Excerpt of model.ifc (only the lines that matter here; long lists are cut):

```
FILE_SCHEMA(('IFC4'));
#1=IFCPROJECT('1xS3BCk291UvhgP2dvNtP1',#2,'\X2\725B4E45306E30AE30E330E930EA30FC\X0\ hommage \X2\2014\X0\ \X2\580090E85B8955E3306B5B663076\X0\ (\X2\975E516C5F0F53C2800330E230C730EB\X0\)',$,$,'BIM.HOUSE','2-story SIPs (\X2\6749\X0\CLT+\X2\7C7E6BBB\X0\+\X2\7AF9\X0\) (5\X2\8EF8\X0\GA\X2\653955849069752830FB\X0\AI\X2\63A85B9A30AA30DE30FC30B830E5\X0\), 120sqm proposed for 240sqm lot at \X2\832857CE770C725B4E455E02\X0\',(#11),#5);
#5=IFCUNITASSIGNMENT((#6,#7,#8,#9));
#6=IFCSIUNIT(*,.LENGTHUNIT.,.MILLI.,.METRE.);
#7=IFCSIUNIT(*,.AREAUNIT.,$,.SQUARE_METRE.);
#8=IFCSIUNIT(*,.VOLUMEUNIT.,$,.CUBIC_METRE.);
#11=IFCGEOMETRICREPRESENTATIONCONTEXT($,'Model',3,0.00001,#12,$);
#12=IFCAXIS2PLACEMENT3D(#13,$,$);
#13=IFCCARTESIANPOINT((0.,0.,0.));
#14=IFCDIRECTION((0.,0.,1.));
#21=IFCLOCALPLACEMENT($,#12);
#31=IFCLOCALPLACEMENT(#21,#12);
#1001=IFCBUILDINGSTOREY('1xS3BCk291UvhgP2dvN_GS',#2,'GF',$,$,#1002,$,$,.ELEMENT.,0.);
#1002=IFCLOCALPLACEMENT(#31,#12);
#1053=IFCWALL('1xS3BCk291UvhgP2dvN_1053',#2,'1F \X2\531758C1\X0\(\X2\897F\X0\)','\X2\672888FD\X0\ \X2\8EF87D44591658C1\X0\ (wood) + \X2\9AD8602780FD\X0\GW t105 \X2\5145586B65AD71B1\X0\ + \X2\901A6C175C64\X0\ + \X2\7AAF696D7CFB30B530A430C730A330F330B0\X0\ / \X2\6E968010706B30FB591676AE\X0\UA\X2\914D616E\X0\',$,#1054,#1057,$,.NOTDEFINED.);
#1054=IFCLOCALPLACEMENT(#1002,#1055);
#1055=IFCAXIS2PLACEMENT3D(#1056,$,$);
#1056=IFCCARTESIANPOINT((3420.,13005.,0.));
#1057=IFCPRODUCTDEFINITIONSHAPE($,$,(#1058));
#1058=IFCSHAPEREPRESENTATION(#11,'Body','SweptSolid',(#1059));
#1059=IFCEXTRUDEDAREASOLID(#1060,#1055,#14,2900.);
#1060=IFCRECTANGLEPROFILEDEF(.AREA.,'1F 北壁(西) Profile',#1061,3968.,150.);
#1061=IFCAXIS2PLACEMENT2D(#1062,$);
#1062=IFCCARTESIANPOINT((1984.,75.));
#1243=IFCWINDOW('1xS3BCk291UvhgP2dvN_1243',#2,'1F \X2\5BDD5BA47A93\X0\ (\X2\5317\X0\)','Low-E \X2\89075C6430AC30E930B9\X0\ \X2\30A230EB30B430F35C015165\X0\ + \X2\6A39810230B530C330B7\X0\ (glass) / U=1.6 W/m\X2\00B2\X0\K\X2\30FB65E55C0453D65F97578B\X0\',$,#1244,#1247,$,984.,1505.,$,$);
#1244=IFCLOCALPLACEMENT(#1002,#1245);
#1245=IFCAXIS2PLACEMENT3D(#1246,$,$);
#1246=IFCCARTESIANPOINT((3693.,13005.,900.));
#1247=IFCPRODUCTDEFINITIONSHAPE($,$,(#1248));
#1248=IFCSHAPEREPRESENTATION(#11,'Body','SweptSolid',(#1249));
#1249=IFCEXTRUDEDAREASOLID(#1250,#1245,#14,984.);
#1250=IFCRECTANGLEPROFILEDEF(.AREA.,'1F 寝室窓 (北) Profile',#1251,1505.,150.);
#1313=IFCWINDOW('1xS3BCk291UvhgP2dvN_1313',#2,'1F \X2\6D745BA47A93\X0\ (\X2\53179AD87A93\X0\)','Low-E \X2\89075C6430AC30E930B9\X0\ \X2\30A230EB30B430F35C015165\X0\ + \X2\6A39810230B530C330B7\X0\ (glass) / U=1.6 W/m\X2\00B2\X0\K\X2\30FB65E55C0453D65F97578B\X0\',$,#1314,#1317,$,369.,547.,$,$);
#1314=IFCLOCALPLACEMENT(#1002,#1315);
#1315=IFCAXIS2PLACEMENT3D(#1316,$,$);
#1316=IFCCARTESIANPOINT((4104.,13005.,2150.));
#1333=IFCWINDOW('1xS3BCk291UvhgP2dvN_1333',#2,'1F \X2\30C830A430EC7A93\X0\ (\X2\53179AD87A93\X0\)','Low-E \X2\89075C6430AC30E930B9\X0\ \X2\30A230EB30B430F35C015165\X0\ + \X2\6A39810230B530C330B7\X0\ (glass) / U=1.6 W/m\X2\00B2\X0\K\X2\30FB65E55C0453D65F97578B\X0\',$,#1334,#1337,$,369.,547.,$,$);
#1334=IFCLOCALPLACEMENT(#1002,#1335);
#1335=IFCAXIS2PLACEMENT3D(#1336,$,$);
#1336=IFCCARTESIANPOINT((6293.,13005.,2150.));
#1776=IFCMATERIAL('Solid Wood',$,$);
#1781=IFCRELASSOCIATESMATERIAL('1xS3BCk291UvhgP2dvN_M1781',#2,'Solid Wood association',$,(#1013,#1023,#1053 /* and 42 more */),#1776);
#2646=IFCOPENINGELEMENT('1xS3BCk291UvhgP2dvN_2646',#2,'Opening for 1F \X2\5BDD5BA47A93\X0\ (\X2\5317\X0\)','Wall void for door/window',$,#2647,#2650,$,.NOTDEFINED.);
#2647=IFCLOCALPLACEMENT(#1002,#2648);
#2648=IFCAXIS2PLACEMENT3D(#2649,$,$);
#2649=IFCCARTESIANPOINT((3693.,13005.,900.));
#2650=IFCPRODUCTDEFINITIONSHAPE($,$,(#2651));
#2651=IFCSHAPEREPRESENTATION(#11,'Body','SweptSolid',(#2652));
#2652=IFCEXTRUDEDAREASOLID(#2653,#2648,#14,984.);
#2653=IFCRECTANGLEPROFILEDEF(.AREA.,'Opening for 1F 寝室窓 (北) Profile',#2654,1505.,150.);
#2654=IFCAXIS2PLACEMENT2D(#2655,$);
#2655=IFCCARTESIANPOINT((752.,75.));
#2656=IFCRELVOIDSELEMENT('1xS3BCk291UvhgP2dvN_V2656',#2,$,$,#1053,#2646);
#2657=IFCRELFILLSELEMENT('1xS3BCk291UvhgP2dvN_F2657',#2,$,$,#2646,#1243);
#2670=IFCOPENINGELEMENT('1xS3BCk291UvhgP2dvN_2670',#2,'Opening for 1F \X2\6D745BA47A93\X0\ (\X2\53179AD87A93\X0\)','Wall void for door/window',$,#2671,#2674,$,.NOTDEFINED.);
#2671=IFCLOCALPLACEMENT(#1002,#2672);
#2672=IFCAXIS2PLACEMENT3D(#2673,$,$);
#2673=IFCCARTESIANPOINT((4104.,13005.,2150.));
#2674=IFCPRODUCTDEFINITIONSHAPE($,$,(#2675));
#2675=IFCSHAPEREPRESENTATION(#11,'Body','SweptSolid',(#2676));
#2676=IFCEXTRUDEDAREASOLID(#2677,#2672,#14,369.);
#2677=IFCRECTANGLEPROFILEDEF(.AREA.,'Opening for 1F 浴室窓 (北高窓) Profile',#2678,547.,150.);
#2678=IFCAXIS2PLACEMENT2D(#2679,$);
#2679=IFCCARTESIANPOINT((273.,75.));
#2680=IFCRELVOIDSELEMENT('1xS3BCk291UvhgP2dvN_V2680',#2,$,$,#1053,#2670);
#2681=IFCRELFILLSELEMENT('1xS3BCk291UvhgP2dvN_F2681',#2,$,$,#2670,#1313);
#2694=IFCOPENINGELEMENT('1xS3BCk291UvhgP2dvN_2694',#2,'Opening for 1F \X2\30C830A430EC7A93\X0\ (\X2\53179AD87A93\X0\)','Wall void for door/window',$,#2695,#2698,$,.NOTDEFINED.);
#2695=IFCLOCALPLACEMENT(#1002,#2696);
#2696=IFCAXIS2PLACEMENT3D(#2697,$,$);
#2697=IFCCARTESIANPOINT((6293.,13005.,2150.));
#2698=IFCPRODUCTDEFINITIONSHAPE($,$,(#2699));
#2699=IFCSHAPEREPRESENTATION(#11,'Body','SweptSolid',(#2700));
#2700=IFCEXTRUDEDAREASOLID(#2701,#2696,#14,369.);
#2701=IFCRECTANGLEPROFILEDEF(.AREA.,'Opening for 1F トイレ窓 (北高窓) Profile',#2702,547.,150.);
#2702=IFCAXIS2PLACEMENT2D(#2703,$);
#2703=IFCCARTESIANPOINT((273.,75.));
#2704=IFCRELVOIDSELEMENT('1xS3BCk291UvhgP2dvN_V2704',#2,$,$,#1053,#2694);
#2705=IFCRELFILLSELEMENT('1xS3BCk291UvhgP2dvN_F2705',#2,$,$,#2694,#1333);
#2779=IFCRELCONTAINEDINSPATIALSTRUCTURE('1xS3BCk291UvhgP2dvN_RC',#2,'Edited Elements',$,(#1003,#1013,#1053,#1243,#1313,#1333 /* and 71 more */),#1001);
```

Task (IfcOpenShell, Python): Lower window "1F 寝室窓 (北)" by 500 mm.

```python
import numpy as np
import ifcopenshell
import ifcopenshell.api.geometry
import ifcopenshell.util.placement
import ifcopenshell.util.unit

model = ifcopenshell.open("model.ifc")
unit_scale = ifcopenshell.util.unit.calculate_unit_scale(model)

window = model.by_guid("1xS3BCk291UvhgP2dvN_1243")
opening = window.FillsVoids[0].RelatingOpeningElement
dz = -500.0

shift = np.array([0.0, 0.0, dz])
# The window is not placed relative to its opening, so move both.
for product in (opening, window):
    matrix = ifcopenshell.util.placement.get_local_placement(product.ObjectPlacement)
    matrix[:3, 3] += shift
    ifcopenshell.api.geometry.edit_object_placement(model, product=product, matrix=matrix, is_si=False)

print(f"moved by {dz * unit_scale:+.3f} m")

model.write("model_edited.ifc")
```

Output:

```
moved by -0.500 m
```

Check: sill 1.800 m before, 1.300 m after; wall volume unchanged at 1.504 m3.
